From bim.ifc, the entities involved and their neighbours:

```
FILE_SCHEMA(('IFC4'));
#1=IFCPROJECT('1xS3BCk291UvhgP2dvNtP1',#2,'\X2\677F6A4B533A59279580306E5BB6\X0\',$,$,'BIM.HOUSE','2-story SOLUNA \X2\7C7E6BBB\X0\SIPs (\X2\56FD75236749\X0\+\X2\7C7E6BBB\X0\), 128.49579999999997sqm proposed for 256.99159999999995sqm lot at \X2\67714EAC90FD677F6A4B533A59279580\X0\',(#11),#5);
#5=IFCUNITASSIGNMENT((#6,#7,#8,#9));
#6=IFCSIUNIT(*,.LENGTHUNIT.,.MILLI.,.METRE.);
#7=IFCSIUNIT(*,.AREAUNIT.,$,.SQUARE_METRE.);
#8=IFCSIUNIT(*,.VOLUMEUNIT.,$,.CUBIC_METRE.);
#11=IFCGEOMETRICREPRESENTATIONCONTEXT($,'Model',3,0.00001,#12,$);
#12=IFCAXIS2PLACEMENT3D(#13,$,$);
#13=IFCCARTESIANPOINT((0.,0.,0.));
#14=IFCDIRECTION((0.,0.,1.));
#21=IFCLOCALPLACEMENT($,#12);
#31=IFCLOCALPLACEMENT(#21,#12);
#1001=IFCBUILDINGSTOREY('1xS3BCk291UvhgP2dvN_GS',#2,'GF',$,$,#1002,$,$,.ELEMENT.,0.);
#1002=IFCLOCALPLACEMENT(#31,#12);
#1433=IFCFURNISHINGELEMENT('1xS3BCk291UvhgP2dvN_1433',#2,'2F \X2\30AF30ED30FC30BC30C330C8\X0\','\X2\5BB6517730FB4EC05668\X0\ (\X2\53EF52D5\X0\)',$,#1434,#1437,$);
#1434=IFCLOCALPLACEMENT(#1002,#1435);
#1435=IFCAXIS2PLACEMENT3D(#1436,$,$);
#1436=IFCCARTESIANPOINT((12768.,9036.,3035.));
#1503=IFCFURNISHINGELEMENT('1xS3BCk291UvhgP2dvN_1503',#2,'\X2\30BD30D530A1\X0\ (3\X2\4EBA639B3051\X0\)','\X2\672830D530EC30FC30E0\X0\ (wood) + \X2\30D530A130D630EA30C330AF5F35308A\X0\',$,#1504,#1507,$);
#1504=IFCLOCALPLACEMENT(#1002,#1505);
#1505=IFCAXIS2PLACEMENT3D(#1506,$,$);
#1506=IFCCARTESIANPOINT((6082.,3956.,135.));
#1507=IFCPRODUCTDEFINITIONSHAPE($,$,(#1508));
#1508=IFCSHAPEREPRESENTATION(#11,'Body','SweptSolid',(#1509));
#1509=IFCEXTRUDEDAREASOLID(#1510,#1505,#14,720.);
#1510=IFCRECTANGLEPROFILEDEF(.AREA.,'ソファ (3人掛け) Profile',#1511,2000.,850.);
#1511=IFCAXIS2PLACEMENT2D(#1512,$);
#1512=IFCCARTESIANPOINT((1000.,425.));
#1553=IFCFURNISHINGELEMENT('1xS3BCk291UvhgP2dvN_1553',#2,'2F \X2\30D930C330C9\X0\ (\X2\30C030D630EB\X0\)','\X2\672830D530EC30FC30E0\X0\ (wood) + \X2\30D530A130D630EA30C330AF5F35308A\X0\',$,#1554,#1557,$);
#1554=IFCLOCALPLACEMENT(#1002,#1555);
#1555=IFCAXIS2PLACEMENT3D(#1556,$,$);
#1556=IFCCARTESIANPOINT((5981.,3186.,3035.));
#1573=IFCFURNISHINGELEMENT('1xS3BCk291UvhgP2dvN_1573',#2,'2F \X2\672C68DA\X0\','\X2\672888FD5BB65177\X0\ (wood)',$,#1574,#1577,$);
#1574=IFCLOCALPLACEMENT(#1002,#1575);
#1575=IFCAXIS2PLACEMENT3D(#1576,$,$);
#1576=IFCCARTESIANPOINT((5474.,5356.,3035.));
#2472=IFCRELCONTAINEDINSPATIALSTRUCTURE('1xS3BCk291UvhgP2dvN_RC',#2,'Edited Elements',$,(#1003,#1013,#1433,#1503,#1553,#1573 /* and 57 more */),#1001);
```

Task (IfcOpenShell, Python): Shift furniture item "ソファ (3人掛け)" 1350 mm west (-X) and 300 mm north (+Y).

```python
import ifcopenshell
import ifcopenshell.api.geometry
import ifcopenshell.util.placement

model = ifcopenshell.open("bim.ifc")

item = model.by_id(1503)
matrix = ifcopenshell.util.placement.get_local_placement(item.ObjectPlacement)
matrix[0, 3] -= 1350.0
matrix[1, 3] += 300.0
ifcopenshell.api.geometry.edit_object_placement(model, product=item, matrix=matrix, is_si=False)

print(ifcopenshell.util.placement.get_local_placement(item.ObjectPlacement).round(3) + 0.0)

model.write("bim_updated.ifc")
```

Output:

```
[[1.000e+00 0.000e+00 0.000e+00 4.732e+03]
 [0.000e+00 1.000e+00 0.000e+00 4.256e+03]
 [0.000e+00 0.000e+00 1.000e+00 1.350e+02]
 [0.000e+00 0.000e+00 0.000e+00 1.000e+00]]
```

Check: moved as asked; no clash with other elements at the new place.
